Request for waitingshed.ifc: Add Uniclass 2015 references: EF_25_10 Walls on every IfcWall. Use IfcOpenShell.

First a look at what the model holds.

```python
import ifcopenshell

model = ifcopenshell.open("waitingshed.ifc")
print(model.schema)
print("classifications:", [c.Name for c in model.by_type("IfcClassification")])
for ifc_class in ("IfcDoor", "IfcRoof", "IfcStair", "IfcWall", "IfcWindow"):
    print(ifc_class, len(model.by_type(ifc_class)))
```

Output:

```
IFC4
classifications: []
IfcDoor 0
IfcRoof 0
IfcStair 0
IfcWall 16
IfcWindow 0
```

```python
import ifcopenshell
import ifcopenshell.api.classification

model = ifcopenshell.open("waitingshed.ifc")

system = ifcopenshell.api.classification.add_classification(model, classification="Uniclass 2015")

codes = {
    "IfcWall": ("EF_25_10", "Walls"),
}
for ifc_class, (code, name) in codes.items():
    products = model.by_type(ifc_class)
    ifcopenshell.api.classification.add_reference(
        model, products=products, classification=system, identification=code, name=name
    )
    print(code, len(products))

model.write("waitingshed_updated.ifc")
```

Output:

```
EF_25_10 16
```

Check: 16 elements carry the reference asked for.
